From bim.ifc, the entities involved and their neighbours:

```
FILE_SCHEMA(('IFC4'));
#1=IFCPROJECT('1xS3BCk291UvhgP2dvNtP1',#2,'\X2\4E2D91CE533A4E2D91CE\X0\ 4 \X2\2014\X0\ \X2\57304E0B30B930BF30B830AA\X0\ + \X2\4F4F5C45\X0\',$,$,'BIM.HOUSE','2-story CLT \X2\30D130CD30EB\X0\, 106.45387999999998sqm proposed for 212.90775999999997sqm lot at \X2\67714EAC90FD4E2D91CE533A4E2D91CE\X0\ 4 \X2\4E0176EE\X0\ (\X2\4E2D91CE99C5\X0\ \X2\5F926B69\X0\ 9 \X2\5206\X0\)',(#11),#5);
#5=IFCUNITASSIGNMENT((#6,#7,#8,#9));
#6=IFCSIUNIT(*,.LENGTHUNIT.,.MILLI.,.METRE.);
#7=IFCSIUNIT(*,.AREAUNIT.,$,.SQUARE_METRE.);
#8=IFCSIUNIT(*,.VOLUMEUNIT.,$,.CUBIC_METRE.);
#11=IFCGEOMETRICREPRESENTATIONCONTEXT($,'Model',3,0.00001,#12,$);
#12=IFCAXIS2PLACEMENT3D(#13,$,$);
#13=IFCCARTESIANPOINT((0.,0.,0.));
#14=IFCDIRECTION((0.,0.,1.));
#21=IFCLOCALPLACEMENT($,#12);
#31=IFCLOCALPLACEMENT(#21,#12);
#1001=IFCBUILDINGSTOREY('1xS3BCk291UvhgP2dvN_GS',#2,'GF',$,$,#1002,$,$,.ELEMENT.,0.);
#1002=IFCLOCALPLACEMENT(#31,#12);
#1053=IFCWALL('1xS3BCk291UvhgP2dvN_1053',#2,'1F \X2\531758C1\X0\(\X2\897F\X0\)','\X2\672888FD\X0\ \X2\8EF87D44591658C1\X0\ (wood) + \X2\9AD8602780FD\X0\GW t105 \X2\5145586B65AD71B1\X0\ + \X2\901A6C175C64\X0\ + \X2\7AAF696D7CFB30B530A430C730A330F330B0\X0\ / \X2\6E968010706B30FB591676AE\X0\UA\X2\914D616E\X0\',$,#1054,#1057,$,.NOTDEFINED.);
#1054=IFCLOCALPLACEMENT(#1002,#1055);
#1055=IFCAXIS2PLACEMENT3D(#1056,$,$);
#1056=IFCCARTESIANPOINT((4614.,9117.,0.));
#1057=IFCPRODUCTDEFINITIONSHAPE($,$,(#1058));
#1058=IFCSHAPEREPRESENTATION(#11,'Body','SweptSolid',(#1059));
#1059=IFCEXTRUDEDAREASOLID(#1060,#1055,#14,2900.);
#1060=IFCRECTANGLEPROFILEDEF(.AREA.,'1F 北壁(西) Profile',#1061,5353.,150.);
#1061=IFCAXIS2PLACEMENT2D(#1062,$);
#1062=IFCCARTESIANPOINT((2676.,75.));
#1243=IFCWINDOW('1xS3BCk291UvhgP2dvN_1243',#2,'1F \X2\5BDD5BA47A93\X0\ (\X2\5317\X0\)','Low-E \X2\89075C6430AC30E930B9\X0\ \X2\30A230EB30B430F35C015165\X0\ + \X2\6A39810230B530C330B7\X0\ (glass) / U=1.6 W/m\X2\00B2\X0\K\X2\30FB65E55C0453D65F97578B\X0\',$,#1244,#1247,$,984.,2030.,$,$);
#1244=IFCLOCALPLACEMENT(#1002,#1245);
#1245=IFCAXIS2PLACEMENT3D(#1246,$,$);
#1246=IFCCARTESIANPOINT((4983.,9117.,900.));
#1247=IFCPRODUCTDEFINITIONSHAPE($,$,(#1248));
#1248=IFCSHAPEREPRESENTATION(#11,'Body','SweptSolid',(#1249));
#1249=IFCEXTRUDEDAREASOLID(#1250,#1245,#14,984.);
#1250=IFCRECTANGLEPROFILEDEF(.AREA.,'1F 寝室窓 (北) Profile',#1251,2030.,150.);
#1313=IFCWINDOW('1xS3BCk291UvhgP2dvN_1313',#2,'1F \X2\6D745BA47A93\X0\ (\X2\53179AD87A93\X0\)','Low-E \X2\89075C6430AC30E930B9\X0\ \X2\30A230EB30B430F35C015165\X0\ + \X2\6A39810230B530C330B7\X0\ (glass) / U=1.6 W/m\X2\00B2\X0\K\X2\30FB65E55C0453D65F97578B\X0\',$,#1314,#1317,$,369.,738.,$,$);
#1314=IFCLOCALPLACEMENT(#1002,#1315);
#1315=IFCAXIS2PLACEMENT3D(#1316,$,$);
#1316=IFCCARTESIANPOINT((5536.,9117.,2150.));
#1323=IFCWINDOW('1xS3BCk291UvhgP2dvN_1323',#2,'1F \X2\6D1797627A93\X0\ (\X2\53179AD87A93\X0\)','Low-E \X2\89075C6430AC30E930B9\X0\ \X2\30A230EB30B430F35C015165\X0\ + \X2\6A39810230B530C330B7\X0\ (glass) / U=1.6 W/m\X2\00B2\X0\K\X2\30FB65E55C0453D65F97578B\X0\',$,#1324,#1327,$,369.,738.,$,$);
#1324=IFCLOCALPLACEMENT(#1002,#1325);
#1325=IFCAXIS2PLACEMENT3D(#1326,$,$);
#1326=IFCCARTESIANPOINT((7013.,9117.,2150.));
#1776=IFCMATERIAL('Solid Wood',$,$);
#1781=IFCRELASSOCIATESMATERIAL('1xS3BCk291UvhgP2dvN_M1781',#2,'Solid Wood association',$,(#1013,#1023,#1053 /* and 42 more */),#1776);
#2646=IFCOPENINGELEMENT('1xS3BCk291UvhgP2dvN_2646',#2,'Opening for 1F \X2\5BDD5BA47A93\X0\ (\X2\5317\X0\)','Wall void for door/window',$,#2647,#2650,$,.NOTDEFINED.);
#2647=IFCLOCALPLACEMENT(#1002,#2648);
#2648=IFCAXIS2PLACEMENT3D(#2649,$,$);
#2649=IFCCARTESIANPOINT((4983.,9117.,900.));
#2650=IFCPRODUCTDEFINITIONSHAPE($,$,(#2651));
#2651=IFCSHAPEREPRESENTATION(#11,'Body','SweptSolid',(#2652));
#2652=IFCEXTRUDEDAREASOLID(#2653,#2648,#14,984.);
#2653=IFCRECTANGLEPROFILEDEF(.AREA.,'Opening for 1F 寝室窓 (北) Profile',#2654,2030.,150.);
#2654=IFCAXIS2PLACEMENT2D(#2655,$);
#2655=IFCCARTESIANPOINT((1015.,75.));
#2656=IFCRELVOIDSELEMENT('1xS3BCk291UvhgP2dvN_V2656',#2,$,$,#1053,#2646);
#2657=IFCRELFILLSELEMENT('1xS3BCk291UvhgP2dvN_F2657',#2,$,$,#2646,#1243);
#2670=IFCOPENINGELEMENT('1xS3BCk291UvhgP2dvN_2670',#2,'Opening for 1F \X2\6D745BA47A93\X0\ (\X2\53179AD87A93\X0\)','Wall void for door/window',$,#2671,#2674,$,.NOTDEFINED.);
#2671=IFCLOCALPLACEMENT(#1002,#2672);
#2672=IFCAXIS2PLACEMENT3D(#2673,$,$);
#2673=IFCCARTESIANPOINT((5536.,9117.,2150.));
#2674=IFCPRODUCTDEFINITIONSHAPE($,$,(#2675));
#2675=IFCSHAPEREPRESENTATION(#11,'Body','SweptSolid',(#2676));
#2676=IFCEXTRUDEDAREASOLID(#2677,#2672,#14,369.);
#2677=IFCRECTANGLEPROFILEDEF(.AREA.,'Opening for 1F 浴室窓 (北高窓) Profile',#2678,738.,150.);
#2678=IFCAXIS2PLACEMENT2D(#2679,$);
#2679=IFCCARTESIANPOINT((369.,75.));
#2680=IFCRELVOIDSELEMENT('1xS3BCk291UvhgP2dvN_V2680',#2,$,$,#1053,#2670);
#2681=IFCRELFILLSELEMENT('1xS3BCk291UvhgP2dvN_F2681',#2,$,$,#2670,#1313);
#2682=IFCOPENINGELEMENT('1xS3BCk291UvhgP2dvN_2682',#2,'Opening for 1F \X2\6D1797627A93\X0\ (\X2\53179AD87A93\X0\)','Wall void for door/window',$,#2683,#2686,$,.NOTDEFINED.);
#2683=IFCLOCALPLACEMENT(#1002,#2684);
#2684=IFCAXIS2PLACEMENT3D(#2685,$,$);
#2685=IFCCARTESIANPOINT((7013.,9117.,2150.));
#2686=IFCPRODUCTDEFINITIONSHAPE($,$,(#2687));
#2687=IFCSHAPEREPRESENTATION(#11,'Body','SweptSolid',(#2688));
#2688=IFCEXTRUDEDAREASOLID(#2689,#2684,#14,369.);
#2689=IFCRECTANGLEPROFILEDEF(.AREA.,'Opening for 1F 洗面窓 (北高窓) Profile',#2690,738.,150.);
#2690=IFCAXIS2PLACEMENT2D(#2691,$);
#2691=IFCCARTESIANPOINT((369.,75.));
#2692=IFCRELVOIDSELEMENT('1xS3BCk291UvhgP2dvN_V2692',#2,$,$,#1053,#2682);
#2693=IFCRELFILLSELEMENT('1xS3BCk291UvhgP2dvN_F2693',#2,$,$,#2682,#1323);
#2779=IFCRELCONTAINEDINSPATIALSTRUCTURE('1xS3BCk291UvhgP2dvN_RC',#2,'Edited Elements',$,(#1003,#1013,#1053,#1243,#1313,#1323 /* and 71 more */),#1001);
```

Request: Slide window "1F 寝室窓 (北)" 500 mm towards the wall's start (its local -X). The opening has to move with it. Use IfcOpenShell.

```python
import ifcopenshell
import ifcopenshell.api.geometry
import ifcopenshell.util.placement

model = ifcopenshell.open("bim.ifc")

window = model.by_guid("1xS3BCk291UvhgP2dvN_1243")
opening = window.FillsVoids[0].RelatingOpeningElement
wall = opening.VoidsElements[0].RelatingBuildingElement

wall_matrix = ifcopenshell.util.placement.get_local_placement(wall.ObjectPlacement)
shift = wall_matrix[:3, 0] * -500.0
before = ifcopenshell.util.placement.get_local_placement(window.ObjectPlacement)[:3, 3].copy()

# The window is not placed relative to its opening, so move both.
for product in (opening, window):
    matrix = ifcopenshell.util.placement.get_local_placement(product.ObjectPlacement)
    matrix[:3, 3] += shift
    ifcopenshell.api.geometry.edit_object_placement(model, product=product, matrix=matrix, is_si=False)

after = ifcopenshell.util.placement.get_local_placement(window.ObjectPlacement)[:3, 3]
print("window moved by", (after - before).round(3) + 0.0)

model.write("bim_rev.ifc")
```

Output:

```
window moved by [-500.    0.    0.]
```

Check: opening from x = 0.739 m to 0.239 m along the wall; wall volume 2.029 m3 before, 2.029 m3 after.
